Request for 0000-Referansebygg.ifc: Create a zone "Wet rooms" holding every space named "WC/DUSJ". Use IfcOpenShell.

First a look at what the model holds.

```python
import ifcopenshell

model = ifcopenshell.open("0000-Referansebygg.ifc")
print(model.schema)
seen = {}
for space in model.by_type("IfcSpace"):
    seen[space.LongName] = seen.get(space.LongName, 0) + 1
for name, count in sorted(seen.items(), key=str):
    print(count, "x", name)
print("zones:", [z.Name for z in model.by_type("IfcZone")][:20])
```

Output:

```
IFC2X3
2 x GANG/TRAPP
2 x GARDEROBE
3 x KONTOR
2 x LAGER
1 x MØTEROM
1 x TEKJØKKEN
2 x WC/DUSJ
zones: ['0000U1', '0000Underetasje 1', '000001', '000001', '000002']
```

```python
import ifcopenshell
import ifcopenshell.api.group
import ifcopenshell.api.root

model = ifcopenshell.open("0000-Referansebygg.ifc")

names = {"WC/DUSJ"}
spaces = [s for s in model.by_type("IfcSpace") if s.LongName in names]

zone = ifcopenshell.api.root.create_entity(model, ifc_class="IfcZone", name="Wet rooms")
ifcopenshell.api.group.assign_group(model, products=spaces, group=zone)
print(len(spaces), "spaces in", zone.Name)

model.write("0000-Referansebygg-out.ifc")
```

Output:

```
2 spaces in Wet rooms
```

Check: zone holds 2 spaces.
